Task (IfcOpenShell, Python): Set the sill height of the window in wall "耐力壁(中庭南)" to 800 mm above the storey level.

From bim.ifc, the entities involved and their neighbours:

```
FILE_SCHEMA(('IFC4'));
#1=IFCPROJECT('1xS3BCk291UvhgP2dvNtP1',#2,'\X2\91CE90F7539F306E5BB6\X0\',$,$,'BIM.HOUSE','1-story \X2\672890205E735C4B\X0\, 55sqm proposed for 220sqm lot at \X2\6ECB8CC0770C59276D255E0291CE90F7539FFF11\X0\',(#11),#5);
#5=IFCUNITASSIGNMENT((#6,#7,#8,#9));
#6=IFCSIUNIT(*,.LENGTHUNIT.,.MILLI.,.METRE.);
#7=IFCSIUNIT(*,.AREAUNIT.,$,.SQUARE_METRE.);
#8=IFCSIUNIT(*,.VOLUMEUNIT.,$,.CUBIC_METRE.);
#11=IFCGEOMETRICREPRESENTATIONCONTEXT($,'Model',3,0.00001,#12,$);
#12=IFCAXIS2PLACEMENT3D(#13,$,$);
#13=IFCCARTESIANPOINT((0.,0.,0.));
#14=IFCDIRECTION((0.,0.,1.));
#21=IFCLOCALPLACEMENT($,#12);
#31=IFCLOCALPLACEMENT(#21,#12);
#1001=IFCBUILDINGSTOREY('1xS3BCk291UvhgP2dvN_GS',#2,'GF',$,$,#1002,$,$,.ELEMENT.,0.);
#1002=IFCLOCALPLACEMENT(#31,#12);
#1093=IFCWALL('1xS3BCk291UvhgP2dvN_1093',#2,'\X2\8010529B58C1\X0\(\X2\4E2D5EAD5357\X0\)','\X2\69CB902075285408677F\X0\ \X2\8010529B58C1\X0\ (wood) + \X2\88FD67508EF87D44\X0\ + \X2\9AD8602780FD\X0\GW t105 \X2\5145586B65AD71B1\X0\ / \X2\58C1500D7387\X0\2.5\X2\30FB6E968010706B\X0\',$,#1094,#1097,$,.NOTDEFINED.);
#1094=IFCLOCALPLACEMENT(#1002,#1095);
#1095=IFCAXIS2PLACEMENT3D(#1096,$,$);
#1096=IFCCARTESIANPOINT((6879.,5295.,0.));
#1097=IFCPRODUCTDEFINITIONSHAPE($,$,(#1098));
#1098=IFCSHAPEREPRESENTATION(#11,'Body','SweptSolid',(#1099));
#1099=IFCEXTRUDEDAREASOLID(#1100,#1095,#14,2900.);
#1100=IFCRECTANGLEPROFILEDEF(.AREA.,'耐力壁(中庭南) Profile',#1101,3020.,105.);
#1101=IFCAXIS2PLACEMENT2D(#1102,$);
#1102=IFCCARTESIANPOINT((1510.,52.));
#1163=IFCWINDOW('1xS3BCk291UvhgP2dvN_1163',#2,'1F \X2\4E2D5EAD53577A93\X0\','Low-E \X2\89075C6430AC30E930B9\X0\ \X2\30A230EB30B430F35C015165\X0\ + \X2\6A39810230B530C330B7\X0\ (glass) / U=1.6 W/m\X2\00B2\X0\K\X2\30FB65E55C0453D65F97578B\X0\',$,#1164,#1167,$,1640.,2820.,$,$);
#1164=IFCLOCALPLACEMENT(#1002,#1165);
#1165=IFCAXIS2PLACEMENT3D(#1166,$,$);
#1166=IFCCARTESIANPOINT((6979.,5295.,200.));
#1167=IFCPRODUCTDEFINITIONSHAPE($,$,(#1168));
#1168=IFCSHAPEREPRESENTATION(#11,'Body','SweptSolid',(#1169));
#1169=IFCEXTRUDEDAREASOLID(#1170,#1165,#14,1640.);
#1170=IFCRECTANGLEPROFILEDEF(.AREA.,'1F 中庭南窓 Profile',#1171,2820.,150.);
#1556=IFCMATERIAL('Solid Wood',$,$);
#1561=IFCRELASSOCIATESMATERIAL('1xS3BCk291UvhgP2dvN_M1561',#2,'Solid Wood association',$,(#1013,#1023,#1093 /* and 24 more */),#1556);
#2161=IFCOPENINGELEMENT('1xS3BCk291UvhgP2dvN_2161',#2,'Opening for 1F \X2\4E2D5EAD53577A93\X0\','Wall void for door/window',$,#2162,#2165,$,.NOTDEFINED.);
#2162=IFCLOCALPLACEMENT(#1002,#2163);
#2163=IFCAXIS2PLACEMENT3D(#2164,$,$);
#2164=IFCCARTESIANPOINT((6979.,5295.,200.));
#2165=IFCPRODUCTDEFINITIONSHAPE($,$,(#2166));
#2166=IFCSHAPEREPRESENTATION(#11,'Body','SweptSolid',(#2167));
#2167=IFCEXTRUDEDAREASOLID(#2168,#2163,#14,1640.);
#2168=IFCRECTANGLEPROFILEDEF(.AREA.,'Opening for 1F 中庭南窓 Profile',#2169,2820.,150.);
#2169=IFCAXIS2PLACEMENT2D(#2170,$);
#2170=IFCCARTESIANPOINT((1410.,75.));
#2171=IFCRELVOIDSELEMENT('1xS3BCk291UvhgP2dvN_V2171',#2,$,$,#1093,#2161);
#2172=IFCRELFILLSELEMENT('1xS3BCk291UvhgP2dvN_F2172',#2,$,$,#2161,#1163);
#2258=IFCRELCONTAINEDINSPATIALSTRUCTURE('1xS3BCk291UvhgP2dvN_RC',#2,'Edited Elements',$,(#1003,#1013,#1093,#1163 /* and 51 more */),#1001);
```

```python
import numpy as np
import ifcopenshell
import ifcopenshell.api.geometry
import ifcopenshell.geom
import ifcopenshell.util.element
import ifcopenshell.util.placement
import ifcopenshell.util.shape
import ifcopenshell.util.unit

model = ifcopenshell.open("bim.ifc")
unit_scale = ifcopenshell.util.unit.calculate_unit_scale(model)

window = model.by_guid("1xS3BCk291UvhgP2dvN_1163")
opening = window.FillsVoids[0].RelatingOpeningElement
storey = ifcopenshell.util.element.get_container(window, ifc_class="IfcBuildingStorey")
level = ifcopenshell.util.placement.get_local_placement(storey.ObjectPlacement)[2, 3]

# The opening's origin need not be at the sill, so measure its lowest point.
shape = ifcopenshell.geom.create_shape(ifcopenshell.geom.settings(), opening)
bottom = ifcopenshell.util.shape.get_shape_bottom_elevation(shape, shape.geometry) / unit_scale
dz = level + 0.8 / unit_scale - bottom

shift = np.array([0.0, 0.0, dz])
# The window is not placed relative to its opening, so move both.
for product in (opening, window):
    matrix = ifcopenshell.util.placement.get_local_placement(product.ObjectPlacement)
    matrix[:3, 3] += shift
    ifcopenshell.api.geometry.edit_object_placement(model, product=product, matrix=matrix, is_si=False)

print(f"moved by {dz * unit_scale:+.3f} m")

model.write("bim_updated.ifc")
```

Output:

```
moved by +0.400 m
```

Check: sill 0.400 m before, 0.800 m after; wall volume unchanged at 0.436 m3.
